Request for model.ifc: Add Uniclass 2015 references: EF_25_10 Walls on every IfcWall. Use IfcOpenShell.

First a look at what the model holds.

```python
import ifcopenshell

model = ifcopenshell.open("model.ifc")
print(model.schema)
print("classifications:", [c.Name for c in model.by_type("IfcClassification")])
for ifc_class in ("IfcDoor", "IfcRoof", "IfcStair", "IfcWall", "IfcWindow"):
    print(ifc_class, len(model.by_type(ifc_class)))
```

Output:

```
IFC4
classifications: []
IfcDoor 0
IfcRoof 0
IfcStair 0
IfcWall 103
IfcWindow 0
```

```python
import ifcopenshell
import ifcopenshell.api.classification

model = ifcopenshell.open("model.ifc")

system = ifcopenshell.api.classification.add_classification(model, classification="Uniclass 2015")

codes = {
    "IfcWall": ("EF_25_10", "Walls"),
}
for ifc_class, (code, name) in codes.items():
    products = model.by_type(ifc_class)
    ifcopenshell.api.classification.add_reference(
        model, products=products, classification=system, identification=code, name=name
    )
    print(code, len(products))

model.write("model_v2.ifc")
```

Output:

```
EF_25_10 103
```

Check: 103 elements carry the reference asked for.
